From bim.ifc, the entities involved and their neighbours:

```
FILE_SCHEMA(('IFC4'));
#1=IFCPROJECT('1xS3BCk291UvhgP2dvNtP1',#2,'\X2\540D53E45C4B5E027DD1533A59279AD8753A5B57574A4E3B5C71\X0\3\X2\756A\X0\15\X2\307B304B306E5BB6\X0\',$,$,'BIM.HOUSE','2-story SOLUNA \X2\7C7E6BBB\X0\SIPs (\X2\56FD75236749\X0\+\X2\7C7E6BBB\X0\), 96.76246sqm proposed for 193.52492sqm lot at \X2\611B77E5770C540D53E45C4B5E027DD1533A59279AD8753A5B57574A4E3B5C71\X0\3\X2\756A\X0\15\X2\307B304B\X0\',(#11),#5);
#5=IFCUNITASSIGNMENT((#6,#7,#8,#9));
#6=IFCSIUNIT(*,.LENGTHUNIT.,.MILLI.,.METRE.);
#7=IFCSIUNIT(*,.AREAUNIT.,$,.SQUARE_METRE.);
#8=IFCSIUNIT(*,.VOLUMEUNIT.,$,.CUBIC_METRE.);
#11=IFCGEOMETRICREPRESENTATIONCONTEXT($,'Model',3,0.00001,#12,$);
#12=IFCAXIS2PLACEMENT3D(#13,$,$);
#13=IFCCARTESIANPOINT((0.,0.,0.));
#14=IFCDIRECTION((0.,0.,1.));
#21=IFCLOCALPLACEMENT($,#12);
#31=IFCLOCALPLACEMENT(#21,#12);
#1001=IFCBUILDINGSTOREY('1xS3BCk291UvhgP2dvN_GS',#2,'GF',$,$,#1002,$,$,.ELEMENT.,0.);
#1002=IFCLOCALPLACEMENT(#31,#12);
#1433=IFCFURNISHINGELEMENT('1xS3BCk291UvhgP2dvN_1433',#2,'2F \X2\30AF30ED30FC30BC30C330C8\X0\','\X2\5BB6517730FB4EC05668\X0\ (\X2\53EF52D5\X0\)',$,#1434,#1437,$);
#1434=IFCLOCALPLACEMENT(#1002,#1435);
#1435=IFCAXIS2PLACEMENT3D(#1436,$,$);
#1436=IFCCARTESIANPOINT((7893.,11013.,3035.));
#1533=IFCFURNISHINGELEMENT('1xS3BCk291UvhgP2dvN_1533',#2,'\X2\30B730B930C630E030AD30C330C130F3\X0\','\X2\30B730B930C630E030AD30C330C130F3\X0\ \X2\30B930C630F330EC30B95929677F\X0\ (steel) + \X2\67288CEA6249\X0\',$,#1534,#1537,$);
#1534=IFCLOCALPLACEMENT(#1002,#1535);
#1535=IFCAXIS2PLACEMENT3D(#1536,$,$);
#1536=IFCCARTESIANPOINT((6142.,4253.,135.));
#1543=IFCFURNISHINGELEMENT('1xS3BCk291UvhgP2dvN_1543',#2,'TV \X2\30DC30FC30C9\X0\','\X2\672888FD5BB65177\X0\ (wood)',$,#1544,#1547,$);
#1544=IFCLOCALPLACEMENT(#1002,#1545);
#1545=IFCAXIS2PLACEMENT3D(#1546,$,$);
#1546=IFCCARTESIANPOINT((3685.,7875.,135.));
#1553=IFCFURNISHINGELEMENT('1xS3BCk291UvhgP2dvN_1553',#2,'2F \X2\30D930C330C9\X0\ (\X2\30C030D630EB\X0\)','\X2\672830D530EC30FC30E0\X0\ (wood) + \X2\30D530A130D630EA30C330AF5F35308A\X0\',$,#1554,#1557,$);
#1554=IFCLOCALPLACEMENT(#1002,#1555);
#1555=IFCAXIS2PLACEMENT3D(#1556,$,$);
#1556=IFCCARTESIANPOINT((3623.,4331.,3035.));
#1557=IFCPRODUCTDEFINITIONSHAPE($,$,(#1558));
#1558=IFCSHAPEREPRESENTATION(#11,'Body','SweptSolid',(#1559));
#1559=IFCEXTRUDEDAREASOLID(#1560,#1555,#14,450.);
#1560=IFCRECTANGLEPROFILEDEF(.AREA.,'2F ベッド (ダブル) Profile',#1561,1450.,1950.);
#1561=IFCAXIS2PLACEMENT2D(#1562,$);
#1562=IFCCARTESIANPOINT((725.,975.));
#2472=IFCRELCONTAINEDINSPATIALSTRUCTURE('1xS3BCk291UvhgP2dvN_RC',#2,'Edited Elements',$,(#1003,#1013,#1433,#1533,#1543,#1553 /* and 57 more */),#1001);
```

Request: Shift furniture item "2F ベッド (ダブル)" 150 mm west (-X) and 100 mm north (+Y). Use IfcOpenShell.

```python
import ifcopenshell
import ifcopenshell.api.geometry
import ifcopenshell.util.placement
import ifcopenshell.util.unit

model = ifcopenshell.open("bim.ifc")
unit_scale = ifcopenshell.util.unit.calculate_unit_scale(model)

item = model.by_guid("1xS3BCk291UvhgP2dvN_1553")
matrix = ifcopenshell.util.placement.get_local_placement(item.ObjectPlacement)
matrix[0, 3] -= 0.15 / unit_scale
matrix[1, 3] += 0.1 / unit_scale
ifcopenshell.api.geometry.edit_object_placement(model, product=item, matrix=matrix, is_si=False)

print(ifcopenshell.util.placement.get_local_placement(item.ObjectPlacement).round(3) + 0.0)

model.write("bim_rev.ifc")
```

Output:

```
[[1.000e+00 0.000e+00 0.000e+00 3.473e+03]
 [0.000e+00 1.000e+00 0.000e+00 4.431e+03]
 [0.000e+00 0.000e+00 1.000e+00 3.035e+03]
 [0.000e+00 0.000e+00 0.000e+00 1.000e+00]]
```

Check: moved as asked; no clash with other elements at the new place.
